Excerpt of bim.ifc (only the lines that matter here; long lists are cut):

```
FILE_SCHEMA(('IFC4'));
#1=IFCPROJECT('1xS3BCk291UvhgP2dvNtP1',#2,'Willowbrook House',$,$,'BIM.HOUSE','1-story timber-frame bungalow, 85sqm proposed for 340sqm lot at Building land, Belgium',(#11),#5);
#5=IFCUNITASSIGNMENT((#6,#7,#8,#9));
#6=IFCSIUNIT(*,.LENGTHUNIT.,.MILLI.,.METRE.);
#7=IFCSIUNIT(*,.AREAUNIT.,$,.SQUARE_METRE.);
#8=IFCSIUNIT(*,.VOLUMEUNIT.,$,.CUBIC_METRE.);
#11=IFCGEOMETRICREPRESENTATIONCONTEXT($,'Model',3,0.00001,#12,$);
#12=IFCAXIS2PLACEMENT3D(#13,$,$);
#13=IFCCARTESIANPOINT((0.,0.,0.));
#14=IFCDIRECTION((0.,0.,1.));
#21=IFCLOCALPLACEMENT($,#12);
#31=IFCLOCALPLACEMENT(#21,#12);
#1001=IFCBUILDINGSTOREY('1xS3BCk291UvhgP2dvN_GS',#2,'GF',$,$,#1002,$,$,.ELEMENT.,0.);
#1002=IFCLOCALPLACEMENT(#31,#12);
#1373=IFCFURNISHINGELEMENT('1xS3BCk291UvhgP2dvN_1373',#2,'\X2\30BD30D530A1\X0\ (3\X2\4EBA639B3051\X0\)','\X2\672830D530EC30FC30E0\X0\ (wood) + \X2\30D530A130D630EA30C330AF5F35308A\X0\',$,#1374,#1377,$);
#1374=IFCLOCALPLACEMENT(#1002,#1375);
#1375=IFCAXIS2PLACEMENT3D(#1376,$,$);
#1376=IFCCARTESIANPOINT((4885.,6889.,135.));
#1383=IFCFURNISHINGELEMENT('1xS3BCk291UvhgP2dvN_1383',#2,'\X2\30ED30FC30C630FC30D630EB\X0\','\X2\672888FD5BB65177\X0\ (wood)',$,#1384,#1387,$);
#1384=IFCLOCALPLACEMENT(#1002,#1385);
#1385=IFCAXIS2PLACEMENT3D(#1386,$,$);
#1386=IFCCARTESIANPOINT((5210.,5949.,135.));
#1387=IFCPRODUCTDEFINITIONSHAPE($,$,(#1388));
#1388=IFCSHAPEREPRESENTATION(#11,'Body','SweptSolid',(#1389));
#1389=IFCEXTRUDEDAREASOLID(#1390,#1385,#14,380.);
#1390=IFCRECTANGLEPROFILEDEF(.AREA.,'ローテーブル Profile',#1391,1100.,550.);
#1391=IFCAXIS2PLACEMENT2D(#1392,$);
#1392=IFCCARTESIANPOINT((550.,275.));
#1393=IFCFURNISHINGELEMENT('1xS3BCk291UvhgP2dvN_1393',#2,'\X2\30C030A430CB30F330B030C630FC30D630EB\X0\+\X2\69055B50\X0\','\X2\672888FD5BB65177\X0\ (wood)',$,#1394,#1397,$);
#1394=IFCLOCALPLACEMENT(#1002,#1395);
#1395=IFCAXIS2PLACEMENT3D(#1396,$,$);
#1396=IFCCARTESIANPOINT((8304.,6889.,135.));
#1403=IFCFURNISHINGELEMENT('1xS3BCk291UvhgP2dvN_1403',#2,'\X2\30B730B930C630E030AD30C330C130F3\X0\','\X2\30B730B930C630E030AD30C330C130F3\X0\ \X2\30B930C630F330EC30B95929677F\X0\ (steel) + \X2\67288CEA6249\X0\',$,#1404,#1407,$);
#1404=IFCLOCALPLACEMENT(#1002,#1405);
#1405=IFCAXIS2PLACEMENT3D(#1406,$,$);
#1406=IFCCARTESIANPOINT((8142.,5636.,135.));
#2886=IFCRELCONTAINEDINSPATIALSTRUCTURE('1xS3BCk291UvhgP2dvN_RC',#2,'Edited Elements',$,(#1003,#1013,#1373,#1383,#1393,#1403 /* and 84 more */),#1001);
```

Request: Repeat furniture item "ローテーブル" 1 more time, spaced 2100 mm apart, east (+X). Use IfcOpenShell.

```python
import numpy as np
import ifcopenshell
import ifcopenshell.api.geometry
import ifcopenshell.api.root
import ifcopenshell.util.element
import ifcopenshell.util.placement
import ifcopenshell.util.unit

model = ifcopenshell.open("bim.ifc")
unit_scale = ifcopenshell.util.unit.calculate_unit_scale(model)


def reuse_history(source, copy):
    """copy_class also copies each property set's owner history, people and application; keep the originals."""
    for rel in copy.IsDefinedBy:
        if rel.is_a("IfcRelDefinesByProperties") and (history := rel.RelatingPropertyDefinition.OwnerHistory):
            rel.RelatingPropertyDefinition.OwnerHistory = source.OwnerHistory
            ifcopenshell.util.element.remove_deep2(model, history)


source = model.by_guid("1xS3BCk291UvhgP2dvN_1383")
base = ifcopenshell.util.placement.get_local_placement(source.ObjectPlacement)
step = np.array([1.0, 0.0, 0.0]) * 2.1 / unit_scale

for i in range(1, 2):
    copy = ifcopenshell.api.root.copy_class(model, product=source)
    copy.Representation = ifcopenshell.util.element.copy_deep(
        model, source.Representation, exclude=["IfcGeometricRepresentationContext", "IfcRepresentationMap"]
    )
    reuse_history(source, copy)
    matrix = base.copy()
    matrix[:3, 3] += i * step
    print("added at", matrix[:3, 3].round(3) + 0.0)
    ifcopenshell.api.geometry.edit_object_placement(model, product=copy, matrix=matrix, is_si=False)

model.write("bim_edited.ifc")
```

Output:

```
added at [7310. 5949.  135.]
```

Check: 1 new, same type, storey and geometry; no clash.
